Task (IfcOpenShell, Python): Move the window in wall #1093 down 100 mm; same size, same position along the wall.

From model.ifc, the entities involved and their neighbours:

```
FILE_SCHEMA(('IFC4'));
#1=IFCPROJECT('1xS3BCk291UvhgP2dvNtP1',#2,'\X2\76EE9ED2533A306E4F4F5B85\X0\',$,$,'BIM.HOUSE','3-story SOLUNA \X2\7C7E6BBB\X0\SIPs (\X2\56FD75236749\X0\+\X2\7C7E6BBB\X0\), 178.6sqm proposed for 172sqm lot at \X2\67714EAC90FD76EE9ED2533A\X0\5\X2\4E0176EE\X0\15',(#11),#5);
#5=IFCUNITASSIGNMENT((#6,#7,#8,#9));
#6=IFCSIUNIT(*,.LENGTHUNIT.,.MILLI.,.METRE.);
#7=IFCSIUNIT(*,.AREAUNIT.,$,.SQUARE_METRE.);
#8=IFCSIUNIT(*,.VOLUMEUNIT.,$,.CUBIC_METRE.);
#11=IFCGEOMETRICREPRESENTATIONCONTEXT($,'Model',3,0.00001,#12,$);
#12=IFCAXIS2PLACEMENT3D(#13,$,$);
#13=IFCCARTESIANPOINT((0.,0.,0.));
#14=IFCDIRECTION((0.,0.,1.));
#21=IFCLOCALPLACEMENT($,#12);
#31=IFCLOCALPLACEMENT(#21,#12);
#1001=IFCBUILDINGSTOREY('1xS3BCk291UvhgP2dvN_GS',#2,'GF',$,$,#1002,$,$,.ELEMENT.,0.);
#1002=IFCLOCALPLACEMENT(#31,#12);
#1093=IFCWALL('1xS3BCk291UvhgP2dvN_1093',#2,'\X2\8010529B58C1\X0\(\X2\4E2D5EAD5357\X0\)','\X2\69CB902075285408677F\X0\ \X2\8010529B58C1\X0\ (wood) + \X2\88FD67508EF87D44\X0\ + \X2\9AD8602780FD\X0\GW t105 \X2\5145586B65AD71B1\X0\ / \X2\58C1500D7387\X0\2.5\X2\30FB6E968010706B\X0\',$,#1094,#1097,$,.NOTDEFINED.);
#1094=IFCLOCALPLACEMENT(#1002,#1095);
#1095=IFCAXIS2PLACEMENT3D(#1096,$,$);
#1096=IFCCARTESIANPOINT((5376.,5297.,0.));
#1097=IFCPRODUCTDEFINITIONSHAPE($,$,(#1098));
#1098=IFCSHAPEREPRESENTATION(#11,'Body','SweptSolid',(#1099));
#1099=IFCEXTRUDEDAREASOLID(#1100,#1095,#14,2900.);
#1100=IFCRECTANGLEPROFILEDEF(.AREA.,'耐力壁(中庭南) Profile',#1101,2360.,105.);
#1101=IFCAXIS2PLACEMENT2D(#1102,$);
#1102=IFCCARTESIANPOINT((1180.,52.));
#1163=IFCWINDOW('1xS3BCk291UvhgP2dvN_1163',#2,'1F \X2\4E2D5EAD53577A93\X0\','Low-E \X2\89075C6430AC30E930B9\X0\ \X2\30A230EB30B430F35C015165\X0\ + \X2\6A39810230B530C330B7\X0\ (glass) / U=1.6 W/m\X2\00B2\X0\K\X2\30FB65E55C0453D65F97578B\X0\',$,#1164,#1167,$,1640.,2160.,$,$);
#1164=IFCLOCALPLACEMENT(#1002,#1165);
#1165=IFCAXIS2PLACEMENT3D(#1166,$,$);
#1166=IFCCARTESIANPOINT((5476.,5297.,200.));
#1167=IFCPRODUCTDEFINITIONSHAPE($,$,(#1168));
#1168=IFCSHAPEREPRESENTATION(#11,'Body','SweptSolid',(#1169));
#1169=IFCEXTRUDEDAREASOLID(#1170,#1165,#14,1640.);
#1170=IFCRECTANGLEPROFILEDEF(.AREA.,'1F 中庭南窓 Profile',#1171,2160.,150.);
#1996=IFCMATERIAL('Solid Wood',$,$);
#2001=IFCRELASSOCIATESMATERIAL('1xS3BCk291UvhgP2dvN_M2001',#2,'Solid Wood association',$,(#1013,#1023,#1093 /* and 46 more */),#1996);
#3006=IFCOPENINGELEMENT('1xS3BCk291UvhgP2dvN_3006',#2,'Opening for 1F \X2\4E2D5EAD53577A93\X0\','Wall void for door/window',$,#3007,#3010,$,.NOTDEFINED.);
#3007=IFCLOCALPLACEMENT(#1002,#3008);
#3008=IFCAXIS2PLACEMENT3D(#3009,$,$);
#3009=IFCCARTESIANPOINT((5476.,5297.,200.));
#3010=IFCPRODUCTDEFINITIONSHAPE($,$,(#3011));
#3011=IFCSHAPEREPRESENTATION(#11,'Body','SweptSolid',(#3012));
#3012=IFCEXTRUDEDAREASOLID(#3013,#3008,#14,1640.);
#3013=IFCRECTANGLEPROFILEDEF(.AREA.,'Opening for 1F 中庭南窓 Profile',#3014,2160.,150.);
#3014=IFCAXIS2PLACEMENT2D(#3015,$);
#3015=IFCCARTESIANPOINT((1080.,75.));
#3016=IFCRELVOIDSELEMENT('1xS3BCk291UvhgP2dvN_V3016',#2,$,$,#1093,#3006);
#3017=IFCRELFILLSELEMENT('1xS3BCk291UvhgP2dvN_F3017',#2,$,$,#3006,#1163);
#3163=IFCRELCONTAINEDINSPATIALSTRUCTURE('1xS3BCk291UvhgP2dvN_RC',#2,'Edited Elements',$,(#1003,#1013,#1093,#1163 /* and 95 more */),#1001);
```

```python
import numpy as np
import ifcopenshell
import ifcopenshell.api.geometry
import ifcopenshell.util.placement
import ifcopenshell.util.unit

model = ifcopenshell.open("model.ifc")
unit_scale = ifcopenshell.util.unit.calculate_unit_scale(model)

window = model.by_id(1163)
opening = window.FillsVoids[0].RelatingOpeningElement
dz = -0.1 / unit_scale

shift = np.array([0.0, 0.0, dz])
# The window is not placed relative to its opening, so move both.
for product in (opening, window):
    matrix = ifcopenshell.util.placement.get_local_placement(product.ObjectPlacement)
    matrix[:3, 3] += shift
    ifcopenshell.api.geometry.edit_object_placement(model, product=product, matrix=matrix, is_si=False)

print(f"moved by {dz * unit_scale:+.3f} m")

model.write("model_updated.ifc")
```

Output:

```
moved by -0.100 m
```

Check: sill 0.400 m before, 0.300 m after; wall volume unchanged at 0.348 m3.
